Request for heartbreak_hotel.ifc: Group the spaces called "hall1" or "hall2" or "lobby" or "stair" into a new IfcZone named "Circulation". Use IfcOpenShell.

First a look at what the model holds.

```python
import ifcopenshell

model = ifcopenshell.open("heartbreak_hotel.ifc")
print(model.schema)
seen = {}
for space in model.by_type("IfcSpace"):
    seen[space.LongName] = seen.get(space.LongName, 0) + 1
for name, count in sorted(seen.items(), key=str):
    print(count, "x", name)
print("zones:", [z.Name for z in model.by_type("IfcZone")][:20])
```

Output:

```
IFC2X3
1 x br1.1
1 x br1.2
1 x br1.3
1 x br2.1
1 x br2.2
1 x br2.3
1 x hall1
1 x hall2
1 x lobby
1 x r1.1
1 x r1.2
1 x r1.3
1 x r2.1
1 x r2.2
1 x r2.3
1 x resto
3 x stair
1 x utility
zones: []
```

```python
import ifcopenshell
import ifcopenshell.api.group
import ifcopenshell.api.root

model = ifcopenshell.open("heartbreak_hotel.ifc")

names = {"hall1", "hall2", "lobby", "stair"}
spaces = [s for s in model.by_type("IfcSpace") if s.LongName in names]

zone = ifcopenshell.api.root.create_entity(model, ifc_class="IfcZone", name="Circulation")
ifcopenshell.api.group.assign_group(model, products=spaces, group=zone)
print(len(spaces), "spaces in", zone.Name)

model.write("heartbreak_hotel_v2.ifc")
```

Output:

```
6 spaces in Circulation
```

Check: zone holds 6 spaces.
